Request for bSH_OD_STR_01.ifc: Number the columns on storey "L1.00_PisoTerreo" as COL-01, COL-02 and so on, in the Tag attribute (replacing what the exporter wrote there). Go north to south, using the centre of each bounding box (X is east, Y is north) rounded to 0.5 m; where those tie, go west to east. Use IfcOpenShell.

First a look at what the model holds.

```python
import ifcopenshell
import ifcopenshell.util.element
import ifcopenshell.util.placement

model = ifcopenshell.open("bSH_OD_STR_01.ifc")
print(model.schema)
storey = next(s for s in model.by_type("IfcBuildingStorey") if s.Name == "L1.00_PisoTerreo")
columns = [e for e in ifcopenshell.util.element.get_decomposition(storey) if e.is_a("IfcColumn")]
for e in sorted(columns, key=lambda e: e.id()):
    origin = ifcopenshell.util.placement.get_local_placement(e.ObjectPlacement)[:3, 3]
    print(e.id(), e.Tag, e.Name, origin.round(2) + 0.0, sep=" | ")
```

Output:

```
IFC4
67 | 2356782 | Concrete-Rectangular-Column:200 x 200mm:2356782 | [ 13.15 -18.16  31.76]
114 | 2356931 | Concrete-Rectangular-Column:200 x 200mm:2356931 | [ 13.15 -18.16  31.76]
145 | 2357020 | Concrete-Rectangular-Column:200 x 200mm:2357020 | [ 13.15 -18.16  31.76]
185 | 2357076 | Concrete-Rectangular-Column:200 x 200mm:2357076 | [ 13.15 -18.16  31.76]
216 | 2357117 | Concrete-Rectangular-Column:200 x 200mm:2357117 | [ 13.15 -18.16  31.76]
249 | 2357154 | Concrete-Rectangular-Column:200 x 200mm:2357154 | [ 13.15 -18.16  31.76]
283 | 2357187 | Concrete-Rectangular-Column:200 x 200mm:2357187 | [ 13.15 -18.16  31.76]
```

```python
import ifcopenshell
import ifcopenshell.geom
import ifcopenshell.util.element
import ifcopenshell.util.shape

model = ifcopenshell.open("bSH_OD_STR_01.ifc")
settings = ifcopenshell.geom.settings()
settings.set("use-world-coords", True)


def centre(element):
    shape = ifcopenshell.geom.create_shape(settings, element)
    return ifcopenshell.util.shape.get_bbox_centroid(shape.geometry)


storey = next(s for s in model.by_type("IfcBuildingStorey") if s.Name == "L1.00_PisoTerreo")
columns = [e for e in ifcopenshell.util.element.get_decomposition(storey) if e.is_a("IfcColumn")]

# Insertion points can sit at a corner or the storey origin, so sort by the geometry (in metres).
centres = {e: centre(e) for e in columns}
columns.sort(key=lambda e: (-round(centres[e][1] / 0.5), centres[e][0]))

for i, e in enumerate(columns, start=1):
    number = f"COL-{i:02d}"
    e.Tag = number
    print(e.id(), number)

model.write("bSH_OD_STR_01_updated.ifc")
```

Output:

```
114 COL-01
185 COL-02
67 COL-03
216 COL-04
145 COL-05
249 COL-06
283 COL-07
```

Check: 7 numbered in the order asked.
